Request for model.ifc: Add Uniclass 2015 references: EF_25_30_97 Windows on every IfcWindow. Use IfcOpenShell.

First a look at what the model holds.

```python
import ifcopenshell

model = ifcopenshell.open("model.ifc")
print(model.schema)
print("classifications:", [c.Name for c in model.by_type("IfcClassification")])
for ifc_class in ("IfcDoor", "IfcRoof", "IfcStair", "IfcWall", "IfcWindow"):
    print(ifc_class, len(model.by_type(ifc_class)))
```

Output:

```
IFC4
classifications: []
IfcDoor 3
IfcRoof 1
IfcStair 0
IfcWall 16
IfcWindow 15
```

```python
import ifcopenshell
import ifcopenshell.api.classification

model = ifcopenshell.open("model.ifc")

system = ifcopenshell.api.classification.add_classification(model, classification="Uniclass 2015")

codes = {
    "IfcWindow": ("EF_25_30_97", "Windows"),
}
for ifc_class, (code, name) in codes.items():
    products = model.by_type(ifc_class)
    ifcopenshell.api.classification.add_reference(
        model, products=products, classification=system, identification=code, name=name
    )
    print(code, len(products))

model.write("model_edited.ifc")
```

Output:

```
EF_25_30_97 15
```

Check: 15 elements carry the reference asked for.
